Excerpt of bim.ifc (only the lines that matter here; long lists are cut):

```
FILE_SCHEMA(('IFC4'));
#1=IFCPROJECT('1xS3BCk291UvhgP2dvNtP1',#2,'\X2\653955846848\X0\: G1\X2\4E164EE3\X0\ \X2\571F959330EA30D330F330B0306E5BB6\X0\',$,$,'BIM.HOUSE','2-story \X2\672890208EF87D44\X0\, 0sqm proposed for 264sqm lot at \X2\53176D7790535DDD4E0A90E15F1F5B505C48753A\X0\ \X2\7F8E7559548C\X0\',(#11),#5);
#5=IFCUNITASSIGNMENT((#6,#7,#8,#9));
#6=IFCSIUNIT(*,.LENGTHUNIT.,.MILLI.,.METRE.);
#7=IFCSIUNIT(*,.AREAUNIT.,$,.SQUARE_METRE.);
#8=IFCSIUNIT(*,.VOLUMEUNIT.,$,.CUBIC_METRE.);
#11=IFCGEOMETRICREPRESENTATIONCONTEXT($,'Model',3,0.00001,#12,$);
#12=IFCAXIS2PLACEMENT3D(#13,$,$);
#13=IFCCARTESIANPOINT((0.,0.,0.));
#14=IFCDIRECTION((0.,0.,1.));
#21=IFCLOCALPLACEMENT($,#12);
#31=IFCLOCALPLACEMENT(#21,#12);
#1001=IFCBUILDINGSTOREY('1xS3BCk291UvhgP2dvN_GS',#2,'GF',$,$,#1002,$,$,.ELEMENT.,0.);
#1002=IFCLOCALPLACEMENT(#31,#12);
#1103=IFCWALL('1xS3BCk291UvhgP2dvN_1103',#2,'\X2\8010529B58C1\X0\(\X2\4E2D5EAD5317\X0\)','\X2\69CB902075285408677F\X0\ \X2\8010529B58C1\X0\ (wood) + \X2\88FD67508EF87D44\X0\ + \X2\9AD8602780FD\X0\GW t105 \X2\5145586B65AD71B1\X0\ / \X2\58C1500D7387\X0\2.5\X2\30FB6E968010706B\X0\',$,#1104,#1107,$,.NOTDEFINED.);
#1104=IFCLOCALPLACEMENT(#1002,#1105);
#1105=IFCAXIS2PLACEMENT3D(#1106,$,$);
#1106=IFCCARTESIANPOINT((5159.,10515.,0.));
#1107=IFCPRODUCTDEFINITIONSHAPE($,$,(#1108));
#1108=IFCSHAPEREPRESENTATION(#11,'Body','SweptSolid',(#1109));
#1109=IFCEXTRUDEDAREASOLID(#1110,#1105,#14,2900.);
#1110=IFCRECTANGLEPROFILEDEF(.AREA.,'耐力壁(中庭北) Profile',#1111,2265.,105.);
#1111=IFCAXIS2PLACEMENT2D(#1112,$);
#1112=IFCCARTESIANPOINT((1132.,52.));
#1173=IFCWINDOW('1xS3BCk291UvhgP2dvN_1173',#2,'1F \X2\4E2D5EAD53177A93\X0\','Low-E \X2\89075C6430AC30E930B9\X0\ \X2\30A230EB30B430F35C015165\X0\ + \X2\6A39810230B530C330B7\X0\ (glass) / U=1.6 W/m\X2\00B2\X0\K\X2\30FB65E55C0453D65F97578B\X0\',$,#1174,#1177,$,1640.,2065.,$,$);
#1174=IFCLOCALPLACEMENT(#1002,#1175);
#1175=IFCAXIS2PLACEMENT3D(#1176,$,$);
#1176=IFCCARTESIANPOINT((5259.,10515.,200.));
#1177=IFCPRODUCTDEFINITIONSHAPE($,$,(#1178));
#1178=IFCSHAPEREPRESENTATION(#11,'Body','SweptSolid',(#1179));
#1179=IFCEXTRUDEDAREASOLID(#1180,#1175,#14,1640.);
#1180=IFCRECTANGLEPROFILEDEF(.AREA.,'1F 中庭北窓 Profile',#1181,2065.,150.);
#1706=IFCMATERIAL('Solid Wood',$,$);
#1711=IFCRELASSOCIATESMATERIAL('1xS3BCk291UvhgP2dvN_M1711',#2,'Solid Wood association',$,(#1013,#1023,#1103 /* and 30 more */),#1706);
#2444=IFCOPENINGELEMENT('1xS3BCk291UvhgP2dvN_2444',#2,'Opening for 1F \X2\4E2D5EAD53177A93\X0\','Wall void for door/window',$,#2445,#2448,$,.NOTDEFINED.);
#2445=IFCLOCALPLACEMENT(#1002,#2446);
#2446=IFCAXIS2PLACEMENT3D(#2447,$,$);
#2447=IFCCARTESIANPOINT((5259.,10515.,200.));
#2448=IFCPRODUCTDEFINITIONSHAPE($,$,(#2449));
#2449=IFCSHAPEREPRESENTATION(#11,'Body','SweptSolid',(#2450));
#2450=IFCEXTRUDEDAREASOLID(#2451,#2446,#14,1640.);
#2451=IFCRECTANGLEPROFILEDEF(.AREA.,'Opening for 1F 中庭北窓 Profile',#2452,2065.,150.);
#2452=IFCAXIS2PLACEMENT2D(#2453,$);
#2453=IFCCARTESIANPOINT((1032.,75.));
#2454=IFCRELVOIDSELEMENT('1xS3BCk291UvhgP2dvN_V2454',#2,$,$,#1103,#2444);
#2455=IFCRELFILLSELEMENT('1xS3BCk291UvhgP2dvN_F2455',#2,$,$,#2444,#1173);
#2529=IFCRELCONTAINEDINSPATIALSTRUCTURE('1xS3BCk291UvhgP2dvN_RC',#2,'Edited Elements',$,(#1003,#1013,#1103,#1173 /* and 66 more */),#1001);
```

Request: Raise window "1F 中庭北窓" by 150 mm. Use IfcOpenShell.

```python
import numpy as np
import ifcopenshell
import ifcopenshell.api.geometry
import ifcopenshell.util.placement
import ifcopenshell.util.unit

model = ifcopenshell.open("bim.ifc")
unit_scale = ifcopenshell.util.unit.calculate_unit_scale(model)

window = model.by_guid("1xS3BCk291UvhgP2dvN_1173")
opening = window.FillsVoids[0].RelatingOpeningElement
dz = 150.0

shift = np.array([0.0, 0.0, dz])
# The window is not placed relative to its opening, so move both.
for product in (opening, window):
    matrix = ifcopenshell.util.placement.get_local_placement(product.ObjectPlacement)
    matrix[:3, 3] += shift
    ifcopenshell.api.geometry.edit_object_placement(model, product=product, matrix=matrix, is_si=False)

print(f"moved by {dz * unit_scale:+.3f} m")

model.write("bim_rev.ifc")
```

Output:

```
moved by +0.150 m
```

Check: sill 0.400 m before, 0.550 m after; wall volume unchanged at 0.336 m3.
